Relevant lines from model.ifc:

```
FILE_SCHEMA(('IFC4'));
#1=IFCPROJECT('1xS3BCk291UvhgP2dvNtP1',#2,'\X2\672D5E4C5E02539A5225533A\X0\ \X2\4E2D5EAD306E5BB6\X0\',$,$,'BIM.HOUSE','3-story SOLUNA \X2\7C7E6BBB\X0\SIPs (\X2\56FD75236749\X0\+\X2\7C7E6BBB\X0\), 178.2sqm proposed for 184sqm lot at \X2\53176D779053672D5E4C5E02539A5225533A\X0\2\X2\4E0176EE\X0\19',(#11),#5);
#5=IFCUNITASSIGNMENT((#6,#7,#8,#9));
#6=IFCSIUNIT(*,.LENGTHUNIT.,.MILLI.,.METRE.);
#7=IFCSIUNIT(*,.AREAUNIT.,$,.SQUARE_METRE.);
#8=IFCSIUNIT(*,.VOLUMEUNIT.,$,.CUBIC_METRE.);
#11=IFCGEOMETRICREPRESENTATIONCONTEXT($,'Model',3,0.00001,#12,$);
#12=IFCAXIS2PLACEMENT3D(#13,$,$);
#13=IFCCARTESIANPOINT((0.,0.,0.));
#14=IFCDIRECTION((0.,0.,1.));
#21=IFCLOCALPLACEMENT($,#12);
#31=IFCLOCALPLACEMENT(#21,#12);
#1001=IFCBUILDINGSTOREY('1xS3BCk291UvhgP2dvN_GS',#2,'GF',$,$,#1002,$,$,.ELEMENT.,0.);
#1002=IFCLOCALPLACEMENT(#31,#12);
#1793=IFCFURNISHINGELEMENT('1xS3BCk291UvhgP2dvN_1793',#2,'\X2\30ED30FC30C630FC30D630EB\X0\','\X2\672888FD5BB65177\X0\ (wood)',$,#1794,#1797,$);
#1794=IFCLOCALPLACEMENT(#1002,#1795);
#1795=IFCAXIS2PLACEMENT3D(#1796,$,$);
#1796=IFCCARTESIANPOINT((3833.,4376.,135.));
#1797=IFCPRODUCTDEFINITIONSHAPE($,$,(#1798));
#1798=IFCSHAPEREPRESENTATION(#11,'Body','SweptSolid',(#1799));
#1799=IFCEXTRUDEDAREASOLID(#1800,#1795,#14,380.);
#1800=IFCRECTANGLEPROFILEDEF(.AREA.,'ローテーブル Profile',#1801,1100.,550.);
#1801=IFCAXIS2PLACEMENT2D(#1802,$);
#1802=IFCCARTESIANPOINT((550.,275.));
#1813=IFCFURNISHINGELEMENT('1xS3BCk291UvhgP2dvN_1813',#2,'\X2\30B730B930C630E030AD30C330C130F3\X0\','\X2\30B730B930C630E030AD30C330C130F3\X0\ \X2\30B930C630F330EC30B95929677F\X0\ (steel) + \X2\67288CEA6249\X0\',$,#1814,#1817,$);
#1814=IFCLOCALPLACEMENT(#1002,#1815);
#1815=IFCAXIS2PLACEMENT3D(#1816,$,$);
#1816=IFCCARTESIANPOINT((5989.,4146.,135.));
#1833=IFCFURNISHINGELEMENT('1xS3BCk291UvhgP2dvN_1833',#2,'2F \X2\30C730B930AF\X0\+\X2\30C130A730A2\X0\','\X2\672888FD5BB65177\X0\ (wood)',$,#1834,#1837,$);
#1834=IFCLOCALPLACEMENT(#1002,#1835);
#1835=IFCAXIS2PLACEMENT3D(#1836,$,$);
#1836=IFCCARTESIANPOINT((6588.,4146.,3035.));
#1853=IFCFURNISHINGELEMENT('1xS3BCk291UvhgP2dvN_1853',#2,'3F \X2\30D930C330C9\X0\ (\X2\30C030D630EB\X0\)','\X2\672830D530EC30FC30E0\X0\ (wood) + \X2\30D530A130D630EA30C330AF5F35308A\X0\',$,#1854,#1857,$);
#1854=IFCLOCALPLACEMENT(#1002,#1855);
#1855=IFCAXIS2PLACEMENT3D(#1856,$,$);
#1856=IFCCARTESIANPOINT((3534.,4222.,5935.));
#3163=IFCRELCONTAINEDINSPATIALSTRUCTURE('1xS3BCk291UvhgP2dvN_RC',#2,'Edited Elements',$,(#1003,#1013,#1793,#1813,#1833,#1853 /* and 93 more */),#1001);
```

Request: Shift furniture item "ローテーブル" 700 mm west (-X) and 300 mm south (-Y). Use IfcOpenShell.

```python
import ifcopenshell
import ifcopenshell.api.geometry
import ifcopenshell.util.placement
import ifcopenshell.util.unit

model = ifcopenshell.open("model.ifc")
unit_scale = ifcopenshell.util.unit.calculate_unit_scale(model)

item = model.by_guid("1xS3BCk291UvhgP2dvN_1793")
matrix = ifcopenshell.util.placement.get_local_placement(item.ObjectPlacement)
matrix[0, 3] -= 0.7 / unit_scale
matrix[1, 3] -= 0.3 / unit_scale
ifcopenshell.api.geometry.edit_object_placement(model, product=item, matrix=matrix, is_si=False)

print(ifcopenshell.util.placement.get_local_placement(item.ObjectPlacement).round(3) + 0.0)

model.write("model_v2.ifc")
```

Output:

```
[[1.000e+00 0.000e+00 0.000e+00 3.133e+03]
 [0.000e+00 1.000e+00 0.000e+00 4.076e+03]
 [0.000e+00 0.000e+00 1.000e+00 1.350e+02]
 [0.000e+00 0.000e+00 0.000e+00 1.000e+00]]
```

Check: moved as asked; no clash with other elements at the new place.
